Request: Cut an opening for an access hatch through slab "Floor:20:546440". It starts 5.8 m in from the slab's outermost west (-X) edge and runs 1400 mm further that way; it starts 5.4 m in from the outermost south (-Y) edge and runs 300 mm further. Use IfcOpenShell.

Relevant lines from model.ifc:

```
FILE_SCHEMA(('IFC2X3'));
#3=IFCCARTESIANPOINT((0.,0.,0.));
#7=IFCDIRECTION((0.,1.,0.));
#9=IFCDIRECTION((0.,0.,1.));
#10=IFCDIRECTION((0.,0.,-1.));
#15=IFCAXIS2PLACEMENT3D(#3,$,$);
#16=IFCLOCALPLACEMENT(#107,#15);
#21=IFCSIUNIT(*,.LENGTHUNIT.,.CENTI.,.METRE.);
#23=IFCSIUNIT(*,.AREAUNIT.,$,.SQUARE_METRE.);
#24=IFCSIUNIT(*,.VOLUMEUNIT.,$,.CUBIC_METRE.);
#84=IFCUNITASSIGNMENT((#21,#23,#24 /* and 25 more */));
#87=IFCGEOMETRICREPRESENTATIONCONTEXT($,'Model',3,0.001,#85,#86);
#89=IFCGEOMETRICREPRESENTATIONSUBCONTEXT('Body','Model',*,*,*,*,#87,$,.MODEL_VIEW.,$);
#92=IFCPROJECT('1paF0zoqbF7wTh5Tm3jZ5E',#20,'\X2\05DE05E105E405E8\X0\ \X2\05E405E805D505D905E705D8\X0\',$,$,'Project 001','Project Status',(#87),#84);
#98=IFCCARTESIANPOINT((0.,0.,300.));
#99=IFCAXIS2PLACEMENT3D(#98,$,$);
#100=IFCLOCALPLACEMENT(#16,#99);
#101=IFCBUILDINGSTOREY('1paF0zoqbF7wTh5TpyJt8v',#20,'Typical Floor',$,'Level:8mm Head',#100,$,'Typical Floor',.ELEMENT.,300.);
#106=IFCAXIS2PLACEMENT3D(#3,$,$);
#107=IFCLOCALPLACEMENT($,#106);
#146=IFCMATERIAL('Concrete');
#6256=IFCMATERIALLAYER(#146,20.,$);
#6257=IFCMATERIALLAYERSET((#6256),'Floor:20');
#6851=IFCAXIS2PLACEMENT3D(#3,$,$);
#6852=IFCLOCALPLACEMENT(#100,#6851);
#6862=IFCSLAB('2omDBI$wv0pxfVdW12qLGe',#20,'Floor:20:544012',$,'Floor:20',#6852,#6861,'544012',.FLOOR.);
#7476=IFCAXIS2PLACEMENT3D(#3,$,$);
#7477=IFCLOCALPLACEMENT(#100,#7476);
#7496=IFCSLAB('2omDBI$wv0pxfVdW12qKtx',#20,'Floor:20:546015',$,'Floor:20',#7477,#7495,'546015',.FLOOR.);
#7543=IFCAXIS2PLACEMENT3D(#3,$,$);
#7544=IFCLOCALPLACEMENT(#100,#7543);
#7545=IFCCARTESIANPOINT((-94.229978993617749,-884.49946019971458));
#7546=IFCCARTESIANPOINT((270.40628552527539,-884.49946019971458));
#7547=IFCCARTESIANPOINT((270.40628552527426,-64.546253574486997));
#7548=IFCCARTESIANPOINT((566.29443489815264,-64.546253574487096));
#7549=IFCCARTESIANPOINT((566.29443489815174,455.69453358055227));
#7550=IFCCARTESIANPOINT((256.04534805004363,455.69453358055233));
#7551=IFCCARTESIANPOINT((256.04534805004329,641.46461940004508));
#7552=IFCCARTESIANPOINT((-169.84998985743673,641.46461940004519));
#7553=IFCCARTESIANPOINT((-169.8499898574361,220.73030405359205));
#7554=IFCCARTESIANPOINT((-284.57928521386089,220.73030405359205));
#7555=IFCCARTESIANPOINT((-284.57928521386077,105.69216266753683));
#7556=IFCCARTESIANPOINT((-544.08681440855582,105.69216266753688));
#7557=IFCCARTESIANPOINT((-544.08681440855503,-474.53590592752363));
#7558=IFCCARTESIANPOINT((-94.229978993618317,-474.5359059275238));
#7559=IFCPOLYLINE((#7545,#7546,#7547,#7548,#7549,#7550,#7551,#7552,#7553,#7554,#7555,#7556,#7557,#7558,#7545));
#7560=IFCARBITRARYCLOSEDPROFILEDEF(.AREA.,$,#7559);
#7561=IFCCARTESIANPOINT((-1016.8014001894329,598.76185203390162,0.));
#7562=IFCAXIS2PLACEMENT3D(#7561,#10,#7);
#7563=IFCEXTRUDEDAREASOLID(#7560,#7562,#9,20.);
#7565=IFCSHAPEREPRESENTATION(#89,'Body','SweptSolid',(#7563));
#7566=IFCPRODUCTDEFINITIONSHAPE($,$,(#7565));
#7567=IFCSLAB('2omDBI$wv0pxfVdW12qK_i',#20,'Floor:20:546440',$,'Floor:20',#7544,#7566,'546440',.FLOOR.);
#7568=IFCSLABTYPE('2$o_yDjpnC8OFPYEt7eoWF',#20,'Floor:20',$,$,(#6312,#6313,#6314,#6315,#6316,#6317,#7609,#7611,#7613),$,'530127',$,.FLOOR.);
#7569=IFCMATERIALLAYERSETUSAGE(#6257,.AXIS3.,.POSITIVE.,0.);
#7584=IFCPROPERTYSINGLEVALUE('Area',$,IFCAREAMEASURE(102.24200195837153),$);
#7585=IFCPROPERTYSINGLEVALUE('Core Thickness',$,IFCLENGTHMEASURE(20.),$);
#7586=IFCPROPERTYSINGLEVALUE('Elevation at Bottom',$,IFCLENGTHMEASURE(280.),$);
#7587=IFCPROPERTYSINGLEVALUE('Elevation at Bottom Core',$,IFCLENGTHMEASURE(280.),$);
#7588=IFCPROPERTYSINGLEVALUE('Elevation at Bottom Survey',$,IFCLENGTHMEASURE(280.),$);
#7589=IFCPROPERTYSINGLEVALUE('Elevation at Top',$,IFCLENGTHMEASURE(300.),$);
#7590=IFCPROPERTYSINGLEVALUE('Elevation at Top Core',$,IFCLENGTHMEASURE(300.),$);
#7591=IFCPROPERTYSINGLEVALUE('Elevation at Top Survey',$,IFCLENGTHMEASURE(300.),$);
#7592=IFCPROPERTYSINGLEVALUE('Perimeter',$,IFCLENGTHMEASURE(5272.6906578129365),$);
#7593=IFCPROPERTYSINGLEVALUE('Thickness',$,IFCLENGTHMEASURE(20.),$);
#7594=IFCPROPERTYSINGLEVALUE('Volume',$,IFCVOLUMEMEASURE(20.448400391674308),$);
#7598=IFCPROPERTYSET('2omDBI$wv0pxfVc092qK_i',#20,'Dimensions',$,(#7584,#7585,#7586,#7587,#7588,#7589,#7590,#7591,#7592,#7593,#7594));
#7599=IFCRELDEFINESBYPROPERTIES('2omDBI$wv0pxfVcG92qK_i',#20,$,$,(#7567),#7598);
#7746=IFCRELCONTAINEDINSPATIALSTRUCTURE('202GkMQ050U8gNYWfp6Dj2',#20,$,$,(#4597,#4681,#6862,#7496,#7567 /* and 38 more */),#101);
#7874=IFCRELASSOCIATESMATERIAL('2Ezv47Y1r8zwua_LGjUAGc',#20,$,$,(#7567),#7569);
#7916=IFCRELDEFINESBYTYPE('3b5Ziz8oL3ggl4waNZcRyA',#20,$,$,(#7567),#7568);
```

```python
import numpy as np
import ifcopenshell
import ifcopenshell.api.feature
import ifcopenshell.api.geometry
import ifcopenshell.api.pset
import ifcopenshell.api.root
import ifcopenshell.geom
import ifcopenshell.util.element
import ifcopenshell.util.placement
import ifcopenshell.util.representation
import ifcopenshell.util.shape
import ifcopenshell.util.unit

model = ifcopenshell.open("model.ifc")
unit_scale = ifcopenshell.util.unit.calculate_unit_scale(model)
area_scale = ifcopenshell.util.unit.calculate_unit_scale(model, "AREAUNIT")
volume_scale = ifcopenshell.util.unit.calculate_unit_scale(model, "VOLUMEUNIT")
settings = ifcopenshell.geom.settings()


def volume(element):
    """Net volume in cubic metres, openings subtracted."""
    shape = ifcopenshell.geom.create_shape(settings, element)
    return ifcopenshell.util.shape.get_volume(shape.geometry)


slab = model.by_guid("2omDBI$wv0pxfVdW12qK_i")
before = volume(slab)

# Extent in the slab's own axes, in metres. The edges named are its -X and -Y sides.
slab_shape = ifcopenshell.geom.create_shape(settings, slab)
vertices = ifcopenshell.util.shape.get_vertices(slab_shape.geometry)
x_min, y_min, bottom = vertices.min(axis=0)
top = vertices[:, 2].max()

opening = ifcopenshell.api.root.create_entity(model, ifc_class="IfcOpeningElement", name="Access hatch opening")
context = ifcopenshell.util.representation.get_context(model, "Model", "Body", "MODEL_VIEW")
width, depth = 1.4, 0.3
outline = [(0.0, 0.0), (width, 0.0), (width, depth), (0.0, depth), (0.0, 0.0)]
# Overshoot both faces by 50 mm so the cut is clean.
shape = ifcopenshell.api.geometry.add_slab_representation(
    model, context=context, depth=top - bottom + 0.1, polyline=outline
)
ifcopenshell.api.geometry.assign_representation(model, product=opening, representation=shape)

matrix = ifcopenshell.util.placement.get_local_placement(slab.ObjectPlacement)
matrix[:, 3] = matrix @ np.append(np.array([x_min + 5.8, y_min + 5.4, bottom - 0.05]) / unit_scale, 1.0)
ifcopenshell.api.geometry.edit_object_placement(model, product=opening, matrix=matrix, is_si=False)
ifcopenshell.api.feature.add_feature(model, feature=opening, element=slab)

after = volume(slab)

# Update the slab's stored quantities.
pset = model.by_id(ifcopenshell.util.element.get_pset(slab, "Dimensions", should_inherit=False)["id"])
ifcopenshell.api.pset.edit_pset(model, pset=pset, properties={
    "Area": model.create_entity("IfcAreaMeasure", after / (top - bottom) / area_scale),
    "Volume": model.create_entity("IfcVolumeMeasure", after / volume_scale),
})

print(f"slab volume {before:.3f} -> {after:.3f} m3")

model.write("model_v2.ifc")
```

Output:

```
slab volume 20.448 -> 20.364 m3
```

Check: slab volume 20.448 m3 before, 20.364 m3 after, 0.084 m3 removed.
